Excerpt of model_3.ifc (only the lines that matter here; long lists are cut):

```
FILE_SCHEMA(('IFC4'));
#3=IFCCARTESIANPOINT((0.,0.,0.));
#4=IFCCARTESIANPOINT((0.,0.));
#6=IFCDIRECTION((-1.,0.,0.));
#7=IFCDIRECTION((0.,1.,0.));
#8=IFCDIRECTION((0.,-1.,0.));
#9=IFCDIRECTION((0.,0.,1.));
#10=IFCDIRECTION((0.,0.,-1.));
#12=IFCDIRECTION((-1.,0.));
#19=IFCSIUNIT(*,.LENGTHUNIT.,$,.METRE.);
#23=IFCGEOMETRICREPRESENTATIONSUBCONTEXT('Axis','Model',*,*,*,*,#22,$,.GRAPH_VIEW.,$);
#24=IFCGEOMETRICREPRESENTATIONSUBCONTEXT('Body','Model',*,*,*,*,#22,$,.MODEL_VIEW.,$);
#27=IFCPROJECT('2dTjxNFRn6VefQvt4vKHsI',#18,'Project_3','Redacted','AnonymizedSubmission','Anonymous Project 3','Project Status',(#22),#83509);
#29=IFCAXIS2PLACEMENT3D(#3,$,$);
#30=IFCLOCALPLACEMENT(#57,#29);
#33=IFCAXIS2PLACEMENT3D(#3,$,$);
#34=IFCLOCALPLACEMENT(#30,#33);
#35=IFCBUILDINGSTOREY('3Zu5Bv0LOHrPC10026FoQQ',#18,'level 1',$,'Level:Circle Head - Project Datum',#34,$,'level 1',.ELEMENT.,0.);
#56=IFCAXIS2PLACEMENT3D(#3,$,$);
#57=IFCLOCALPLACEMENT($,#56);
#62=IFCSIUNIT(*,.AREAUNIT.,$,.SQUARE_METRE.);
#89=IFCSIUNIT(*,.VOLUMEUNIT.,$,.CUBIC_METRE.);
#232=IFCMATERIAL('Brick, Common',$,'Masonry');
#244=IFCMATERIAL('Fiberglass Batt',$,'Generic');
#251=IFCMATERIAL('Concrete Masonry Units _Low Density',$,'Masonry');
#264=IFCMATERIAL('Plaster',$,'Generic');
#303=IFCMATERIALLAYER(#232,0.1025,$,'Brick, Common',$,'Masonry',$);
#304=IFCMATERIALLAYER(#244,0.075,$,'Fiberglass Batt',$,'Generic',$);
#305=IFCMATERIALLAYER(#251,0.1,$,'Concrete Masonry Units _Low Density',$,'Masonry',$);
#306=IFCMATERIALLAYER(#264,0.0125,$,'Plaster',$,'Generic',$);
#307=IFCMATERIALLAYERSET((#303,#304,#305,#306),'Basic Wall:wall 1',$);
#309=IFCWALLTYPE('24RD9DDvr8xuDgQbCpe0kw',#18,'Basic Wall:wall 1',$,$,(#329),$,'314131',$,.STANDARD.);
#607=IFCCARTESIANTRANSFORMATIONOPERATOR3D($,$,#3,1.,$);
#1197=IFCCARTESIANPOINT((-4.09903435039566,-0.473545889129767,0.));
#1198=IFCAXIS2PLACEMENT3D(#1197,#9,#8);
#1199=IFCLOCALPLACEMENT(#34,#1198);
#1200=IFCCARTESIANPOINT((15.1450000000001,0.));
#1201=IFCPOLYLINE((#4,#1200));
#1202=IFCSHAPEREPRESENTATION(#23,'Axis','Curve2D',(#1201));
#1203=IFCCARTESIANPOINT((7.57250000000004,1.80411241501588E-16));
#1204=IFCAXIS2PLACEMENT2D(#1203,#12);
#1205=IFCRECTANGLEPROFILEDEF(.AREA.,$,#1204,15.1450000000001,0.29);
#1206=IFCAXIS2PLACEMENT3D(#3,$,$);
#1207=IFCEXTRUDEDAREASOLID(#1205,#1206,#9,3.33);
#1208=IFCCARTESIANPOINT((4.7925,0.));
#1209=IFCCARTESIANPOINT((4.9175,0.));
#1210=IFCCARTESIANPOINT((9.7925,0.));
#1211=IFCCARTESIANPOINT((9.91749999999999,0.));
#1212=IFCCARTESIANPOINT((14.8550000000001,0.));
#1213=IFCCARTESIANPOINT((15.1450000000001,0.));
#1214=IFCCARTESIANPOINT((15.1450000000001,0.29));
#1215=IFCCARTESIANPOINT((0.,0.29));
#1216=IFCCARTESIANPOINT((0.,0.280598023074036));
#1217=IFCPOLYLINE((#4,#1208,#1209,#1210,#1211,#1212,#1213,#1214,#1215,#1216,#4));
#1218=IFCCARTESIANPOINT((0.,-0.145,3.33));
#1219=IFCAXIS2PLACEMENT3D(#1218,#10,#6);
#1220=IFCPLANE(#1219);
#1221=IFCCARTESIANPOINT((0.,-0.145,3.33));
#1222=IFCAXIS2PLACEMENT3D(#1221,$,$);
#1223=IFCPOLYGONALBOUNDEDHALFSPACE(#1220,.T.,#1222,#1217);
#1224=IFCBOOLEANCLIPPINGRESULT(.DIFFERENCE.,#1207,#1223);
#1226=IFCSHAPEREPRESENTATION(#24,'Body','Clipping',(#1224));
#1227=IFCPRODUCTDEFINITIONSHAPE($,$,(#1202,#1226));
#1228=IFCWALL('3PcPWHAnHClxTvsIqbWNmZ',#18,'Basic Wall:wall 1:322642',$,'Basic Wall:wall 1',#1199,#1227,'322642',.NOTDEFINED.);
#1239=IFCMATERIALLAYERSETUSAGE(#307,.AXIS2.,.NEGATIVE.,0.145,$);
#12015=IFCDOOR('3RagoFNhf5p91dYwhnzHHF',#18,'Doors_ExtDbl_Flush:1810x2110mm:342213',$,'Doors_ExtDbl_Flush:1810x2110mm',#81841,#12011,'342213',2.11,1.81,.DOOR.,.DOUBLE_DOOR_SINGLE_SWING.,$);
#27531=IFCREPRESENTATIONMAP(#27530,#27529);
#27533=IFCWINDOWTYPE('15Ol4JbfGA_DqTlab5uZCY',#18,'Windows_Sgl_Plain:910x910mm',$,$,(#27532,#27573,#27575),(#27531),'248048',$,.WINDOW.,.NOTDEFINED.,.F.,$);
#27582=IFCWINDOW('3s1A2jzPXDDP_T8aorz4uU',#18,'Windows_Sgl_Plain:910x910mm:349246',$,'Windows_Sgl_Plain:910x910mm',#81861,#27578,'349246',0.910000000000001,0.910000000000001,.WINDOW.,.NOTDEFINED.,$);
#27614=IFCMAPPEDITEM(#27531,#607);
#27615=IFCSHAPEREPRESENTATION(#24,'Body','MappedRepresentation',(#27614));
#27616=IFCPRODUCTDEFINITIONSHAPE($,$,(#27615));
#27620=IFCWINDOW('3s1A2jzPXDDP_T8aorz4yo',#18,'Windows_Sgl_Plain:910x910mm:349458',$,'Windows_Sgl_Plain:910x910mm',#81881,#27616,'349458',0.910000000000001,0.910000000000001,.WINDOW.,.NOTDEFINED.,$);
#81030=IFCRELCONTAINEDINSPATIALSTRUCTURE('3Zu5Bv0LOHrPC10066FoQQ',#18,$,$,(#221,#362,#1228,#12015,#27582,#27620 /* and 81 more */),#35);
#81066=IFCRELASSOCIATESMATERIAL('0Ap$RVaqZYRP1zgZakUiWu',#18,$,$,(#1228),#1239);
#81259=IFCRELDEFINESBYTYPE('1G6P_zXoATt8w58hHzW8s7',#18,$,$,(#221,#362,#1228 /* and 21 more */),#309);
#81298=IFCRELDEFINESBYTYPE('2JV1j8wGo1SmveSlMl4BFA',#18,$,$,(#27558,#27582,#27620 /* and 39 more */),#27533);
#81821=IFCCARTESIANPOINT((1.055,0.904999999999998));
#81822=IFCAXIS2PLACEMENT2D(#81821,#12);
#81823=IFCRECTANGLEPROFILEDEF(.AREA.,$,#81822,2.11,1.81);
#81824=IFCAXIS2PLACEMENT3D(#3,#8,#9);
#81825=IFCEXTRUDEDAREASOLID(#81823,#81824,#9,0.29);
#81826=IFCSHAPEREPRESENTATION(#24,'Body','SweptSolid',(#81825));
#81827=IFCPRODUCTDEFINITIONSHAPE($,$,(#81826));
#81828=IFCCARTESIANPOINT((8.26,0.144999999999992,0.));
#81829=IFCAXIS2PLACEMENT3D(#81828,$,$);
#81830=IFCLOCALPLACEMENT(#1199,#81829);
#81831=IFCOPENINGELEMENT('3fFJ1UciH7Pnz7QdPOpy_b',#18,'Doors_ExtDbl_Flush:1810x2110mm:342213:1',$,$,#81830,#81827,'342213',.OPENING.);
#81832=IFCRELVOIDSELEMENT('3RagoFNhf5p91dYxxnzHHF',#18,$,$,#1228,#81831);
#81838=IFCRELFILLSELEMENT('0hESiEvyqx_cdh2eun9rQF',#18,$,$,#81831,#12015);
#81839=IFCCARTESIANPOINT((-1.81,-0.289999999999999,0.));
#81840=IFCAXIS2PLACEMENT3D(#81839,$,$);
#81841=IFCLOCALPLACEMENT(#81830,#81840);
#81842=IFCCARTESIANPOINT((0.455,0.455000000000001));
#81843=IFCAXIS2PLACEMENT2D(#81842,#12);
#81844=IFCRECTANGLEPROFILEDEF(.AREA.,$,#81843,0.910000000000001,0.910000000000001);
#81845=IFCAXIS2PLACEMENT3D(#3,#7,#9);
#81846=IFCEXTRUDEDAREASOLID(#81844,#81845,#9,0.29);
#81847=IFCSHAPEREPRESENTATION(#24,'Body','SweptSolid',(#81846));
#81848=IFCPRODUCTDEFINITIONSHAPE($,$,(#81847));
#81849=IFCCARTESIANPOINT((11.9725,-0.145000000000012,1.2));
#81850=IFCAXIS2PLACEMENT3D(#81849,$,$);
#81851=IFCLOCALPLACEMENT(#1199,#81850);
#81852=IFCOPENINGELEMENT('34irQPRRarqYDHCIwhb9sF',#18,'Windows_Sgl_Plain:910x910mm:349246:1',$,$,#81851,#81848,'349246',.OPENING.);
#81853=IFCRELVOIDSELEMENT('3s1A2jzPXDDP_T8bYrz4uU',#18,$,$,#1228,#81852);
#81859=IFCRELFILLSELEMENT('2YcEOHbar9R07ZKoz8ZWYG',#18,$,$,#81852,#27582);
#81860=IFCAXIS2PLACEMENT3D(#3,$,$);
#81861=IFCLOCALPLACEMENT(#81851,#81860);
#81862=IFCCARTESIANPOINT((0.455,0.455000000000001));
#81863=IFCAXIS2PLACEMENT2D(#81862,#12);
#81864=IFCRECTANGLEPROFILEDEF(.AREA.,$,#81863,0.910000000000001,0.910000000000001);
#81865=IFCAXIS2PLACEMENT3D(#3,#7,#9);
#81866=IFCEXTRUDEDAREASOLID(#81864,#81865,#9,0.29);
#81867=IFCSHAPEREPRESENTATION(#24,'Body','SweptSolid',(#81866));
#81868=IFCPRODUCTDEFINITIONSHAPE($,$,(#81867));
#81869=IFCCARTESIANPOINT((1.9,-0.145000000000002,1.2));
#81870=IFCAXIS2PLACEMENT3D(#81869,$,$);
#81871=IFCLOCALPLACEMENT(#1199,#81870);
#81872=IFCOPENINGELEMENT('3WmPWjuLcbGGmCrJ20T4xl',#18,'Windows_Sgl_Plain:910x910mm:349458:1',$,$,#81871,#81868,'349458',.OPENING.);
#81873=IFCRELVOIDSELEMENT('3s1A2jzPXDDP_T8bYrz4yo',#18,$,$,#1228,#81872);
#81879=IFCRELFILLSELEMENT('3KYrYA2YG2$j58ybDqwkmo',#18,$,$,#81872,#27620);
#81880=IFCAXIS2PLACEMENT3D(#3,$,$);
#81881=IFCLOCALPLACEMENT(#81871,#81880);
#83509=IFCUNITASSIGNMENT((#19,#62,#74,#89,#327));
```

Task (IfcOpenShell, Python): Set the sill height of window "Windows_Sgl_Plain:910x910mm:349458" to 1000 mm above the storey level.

```python
import numpy as np
import ifcopenshell
import ifcopenshell.api.geometry
import ifcopenshell.geom
import ifcopenshell.util.element
import ifcopenshell.util.placement
import ifcopenshell.util.shape
import ifcopenshell.util.unit

model = ifcopenshell.open("model_3.ifc")
unit_scale = ifcopenshell.util.unit.calculate_unit_scale(model)

window = model.by_id(27620)
opening = window.FillsVoids[0].RelatingOpeningElement
storey = ifcopenshell.util.element.get_container(window, ifc_class="IfcBuildingStorey")
level = ifcopenshell.util.placement.get_local_placement(storey.ObjectPlacement)[2, 3]

# The opening's origin need not be at the sill, so measure its lowest point.
shape = ifcopenshell.geom.create_shape(ifcopenshell.geom.settings(), opening)
bottom = ifcopenshell.util.shape.get_shape_bottom_elevation(shape, shape.geometry) / unit_scale
dz = level + 1.0 - bottom

shift = np.array([0.0, 0.0, dz])
# The window is placed relative to its opening, so it follows when the opening moves.
matrix = ifcopenshell.util.placement.get_local_placement(opening.ObjectPlacement)
matrix[:3, 3] += shift
ifcopenshell.api.geometry.edit_object_placement(
    model, product=opening, matrix=matrix, is_si=False, should_transform_children=True
)

print(f"moved by {dz * unit_scale:+.3f} m")

model.write("model_3_updated.ifc")
```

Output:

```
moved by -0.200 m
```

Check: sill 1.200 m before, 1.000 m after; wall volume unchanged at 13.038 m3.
